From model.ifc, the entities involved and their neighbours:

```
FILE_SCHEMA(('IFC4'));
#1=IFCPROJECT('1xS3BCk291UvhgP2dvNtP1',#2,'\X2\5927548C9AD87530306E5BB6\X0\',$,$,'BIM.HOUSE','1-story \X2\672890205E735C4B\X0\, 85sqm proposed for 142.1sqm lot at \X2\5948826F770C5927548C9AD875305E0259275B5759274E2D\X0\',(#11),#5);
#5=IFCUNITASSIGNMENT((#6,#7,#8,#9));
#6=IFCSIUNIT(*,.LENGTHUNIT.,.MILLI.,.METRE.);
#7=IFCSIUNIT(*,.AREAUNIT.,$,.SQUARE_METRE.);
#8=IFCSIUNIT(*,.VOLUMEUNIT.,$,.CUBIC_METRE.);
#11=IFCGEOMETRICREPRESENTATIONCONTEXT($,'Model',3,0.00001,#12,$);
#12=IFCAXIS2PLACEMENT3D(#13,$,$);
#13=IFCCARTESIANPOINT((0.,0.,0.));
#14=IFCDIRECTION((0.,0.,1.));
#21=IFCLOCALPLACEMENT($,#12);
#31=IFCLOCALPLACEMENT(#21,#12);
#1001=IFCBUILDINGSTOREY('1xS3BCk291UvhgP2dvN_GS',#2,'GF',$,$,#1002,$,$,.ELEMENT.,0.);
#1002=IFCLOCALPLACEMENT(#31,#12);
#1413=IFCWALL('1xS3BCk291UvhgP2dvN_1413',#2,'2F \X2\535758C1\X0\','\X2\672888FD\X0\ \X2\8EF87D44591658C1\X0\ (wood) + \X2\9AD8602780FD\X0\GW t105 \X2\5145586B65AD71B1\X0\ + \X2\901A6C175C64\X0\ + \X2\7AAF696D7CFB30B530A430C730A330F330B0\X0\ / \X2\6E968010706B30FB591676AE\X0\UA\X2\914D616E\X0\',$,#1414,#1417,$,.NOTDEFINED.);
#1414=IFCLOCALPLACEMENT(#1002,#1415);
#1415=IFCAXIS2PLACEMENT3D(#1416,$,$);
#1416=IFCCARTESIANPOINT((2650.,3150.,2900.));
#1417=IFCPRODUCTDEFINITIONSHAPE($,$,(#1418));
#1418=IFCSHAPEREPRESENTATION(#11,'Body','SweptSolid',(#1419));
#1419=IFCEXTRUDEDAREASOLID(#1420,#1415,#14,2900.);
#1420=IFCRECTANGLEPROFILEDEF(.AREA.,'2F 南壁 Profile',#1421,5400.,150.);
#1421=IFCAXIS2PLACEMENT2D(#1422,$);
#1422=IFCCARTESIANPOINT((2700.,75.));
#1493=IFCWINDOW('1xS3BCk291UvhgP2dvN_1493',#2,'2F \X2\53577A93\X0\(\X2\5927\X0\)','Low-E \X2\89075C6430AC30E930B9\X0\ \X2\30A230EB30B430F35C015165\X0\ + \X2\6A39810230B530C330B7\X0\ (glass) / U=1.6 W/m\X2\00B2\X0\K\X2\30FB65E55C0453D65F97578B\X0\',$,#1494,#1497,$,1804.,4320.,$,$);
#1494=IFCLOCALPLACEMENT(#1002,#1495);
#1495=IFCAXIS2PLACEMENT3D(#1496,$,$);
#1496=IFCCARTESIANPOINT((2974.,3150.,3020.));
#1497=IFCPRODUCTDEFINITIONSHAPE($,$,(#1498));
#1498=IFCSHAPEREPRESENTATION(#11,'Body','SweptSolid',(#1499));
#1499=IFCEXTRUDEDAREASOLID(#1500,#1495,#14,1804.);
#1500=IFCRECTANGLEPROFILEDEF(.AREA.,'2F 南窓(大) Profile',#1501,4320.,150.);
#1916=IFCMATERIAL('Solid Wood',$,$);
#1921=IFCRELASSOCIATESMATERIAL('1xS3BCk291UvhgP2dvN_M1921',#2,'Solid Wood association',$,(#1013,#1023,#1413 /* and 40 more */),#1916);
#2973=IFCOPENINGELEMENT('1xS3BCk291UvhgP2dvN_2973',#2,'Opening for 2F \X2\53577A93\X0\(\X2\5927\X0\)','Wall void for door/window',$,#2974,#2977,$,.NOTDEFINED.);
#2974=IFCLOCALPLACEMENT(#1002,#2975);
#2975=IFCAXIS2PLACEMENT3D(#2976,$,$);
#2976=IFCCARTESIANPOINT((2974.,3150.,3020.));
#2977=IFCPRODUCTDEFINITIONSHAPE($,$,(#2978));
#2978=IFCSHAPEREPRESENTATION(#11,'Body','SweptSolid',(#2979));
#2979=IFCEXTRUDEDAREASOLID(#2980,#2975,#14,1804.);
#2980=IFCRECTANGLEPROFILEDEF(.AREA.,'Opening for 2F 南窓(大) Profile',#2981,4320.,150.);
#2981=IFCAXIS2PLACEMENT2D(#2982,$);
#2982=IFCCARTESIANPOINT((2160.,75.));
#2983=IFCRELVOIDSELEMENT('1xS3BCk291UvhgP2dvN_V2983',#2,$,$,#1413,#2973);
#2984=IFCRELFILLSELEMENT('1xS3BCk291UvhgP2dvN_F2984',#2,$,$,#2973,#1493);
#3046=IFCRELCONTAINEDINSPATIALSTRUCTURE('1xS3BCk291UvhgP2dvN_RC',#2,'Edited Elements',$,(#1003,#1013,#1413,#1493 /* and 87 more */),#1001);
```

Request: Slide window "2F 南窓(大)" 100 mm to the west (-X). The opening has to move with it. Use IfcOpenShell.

```python
import ifcopenshell
import ifcopenshell.api.geometry
import ifcopenshell.util.placement
import ifcopenshell.util.unit

model = ifcopenshell.open("model.ifc")
unit_scale = ifcopenshell.util.unit.calculate_unit_scale(model)

window = model.by_guid("1xS3BCk291UvhgP2dvN_1493")
opening = window.FillsVoids[0].RelatingOpeningElement
wall = opening.VoidsElements[0].RelatingBuildingElement

wall_matrix = ifcopenshell.util.placement.get_local_placement(wall.ObjectPlacement)
shift = wall_matrix[:3, 0] * -0.1 / unit_scale
before = ifcopenshell.util.placement.get_local_placement(window.ObjectPlacement)[:3, 3].copy()

# The window is not placed relative to its opening, so move both.
for product in (opening, window):
    matrix = ifcopenshell.util.placement.get_local_placement(product.ObjectPlacement)
    matrix[:3, 3] += shift
    ifcopenshell.api.geometry.edit_object_placement(model, product=product, matrix=matrix, is_si=False)

after = ifcopenshell.util.placement.get_local_placement(window.ObjectPlacement)[:3, 3]
print("window moved by", (after - before).round(3) + 0.0)

model.write("model_rev.ifc")
```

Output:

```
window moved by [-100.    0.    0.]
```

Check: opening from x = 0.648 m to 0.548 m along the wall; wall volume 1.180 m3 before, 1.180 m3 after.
